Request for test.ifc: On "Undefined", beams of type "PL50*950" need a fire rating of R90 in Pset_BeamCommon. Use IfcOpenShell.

First a look at what the model holds.

```python
import ifcopenshell
import ifcopenshell.util.element

model = ifcopenshell.open("test.ifc")
print(model.schema)
storey = next(s for s in model.by_type("IfcBuildingStorey") if s.Name == "Undefined")
beams = [e for e in ifcopenshell.util.element.get_decomposition(storey) if e.is_a("IfcBeam")]
seen = {}
for e in beams:
    element_type = ifcopenshell.util.element.get_type(e)
    key = (element_type.Name if element_type != e and element_type else None, ifcopenshell.util.element.get_pset(e, "Pset_BeamCommon", "FireRating"))
    seen[key] = seen.get(key, 0) + 1
for (name, value), count in sorted(seen.items(), key=str):
    print(count, "x", name, "|", value)
```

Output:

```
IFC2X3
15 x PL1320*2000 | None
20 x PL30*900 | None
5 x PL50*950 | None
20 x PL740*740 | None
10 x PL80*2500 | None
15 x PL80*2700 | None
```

```python
import ifcopenshell
import ifcopenshell.api.pset
import ifcopenshell.util.element

model = ifcopenshell.open("test.ifc")

storey = next(s for s in model.by_type("IfcBuildingStorey") if s.Name == "Undefined")
beams = [e for e in ifcopenshell.util.element.get_decomposition(storey) if e.is_a("IfcBeam")]

count = 0
for e in beams:
    element_type = ifcopenshell.util.element.get_type(e)
    if element_type in (None, e) or element_type.Name != "PL50*950":
        continue
    found = ifcopenshell.util.element.get_pset(e, "Pset_BeamCommon", should_inherit=False)
    if found:
        pset = model.by_id(found["id"])
        if len(ifcopenshell.util.element.get_elements_by_pset(pset)) > 1:
            pset = ifcopenshell.api.pset.unshare_pset(model, products=[e], pset=pset)[0]
    else:
        pset = ifcopenshell.api.pset.add_pset(model, product=e, name="Pset_BeamCommon")
    ifcopenshell.api.pset.edit_pset(model, pset=pset, properties={"FireRating": "R90"})
    count += 1

print(count, "beams updated")

model.write("test_rev.ifc")
```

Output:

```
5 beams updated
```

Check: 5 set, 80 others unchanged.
